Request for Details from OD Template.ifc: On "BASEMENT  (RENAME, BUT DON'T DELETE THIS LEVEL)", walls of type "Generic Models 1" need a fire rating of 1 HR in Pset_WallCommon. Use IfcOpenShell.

First a look at what the model holds.

```python
import ifcopenshell
import ifcopenshell.util.element

model = ifcopenshell.open("Details from OD Template.ifc")
print(model.schema)
storey = next(s for s in model.by_type("IfcBuildingStorey") if s.Name == "BASEMENT  (RENAME, BUT DON'T DELETE THIS LEVEL)")
walls = [e for e in ifcopenshell.util.element.get_decomposition(storey) if e.is_a("IfcWall")]
seen = {}
for e in walls:
    element_type = ifcopenshell.util.element.get_type(e)
    key = (element_type.Name if element_type != e and element_type else None, ifcopenshell.util.element.get_pset(e, "Pset_WallCommon", "FireRating"))
    seen[key] = seen.get(key, 0) + 1
for (name, value), count in sorted(seen.items(), key=str):
    print(count, "x", name, "|", value)
```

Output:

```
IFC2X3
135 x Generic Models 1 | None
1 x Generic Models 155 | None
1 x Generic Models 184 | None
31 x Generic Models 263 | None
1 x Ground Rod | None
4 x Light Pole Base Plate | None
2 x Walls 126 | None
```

```python
import ifcopenshell
import ifcopenshell.api.pset
import ifcopenshell.util.element

model = ifcopenshell.open("Details from OD Template.ifc")

storey = next(s for s in model.by_type("IfcBuildingStorey") if s.Name == "BASEMENT  (RENAME, BUT DON'T DELETE THIS LEVEL)")
walls = [e for e in ifcopenshell.util.element.get_decomposition(storey) if e.is_a("IfcWall")]

count = 0
for e in walls:
    element_type = ifcopenshell.util.element.get_type(e)
    if element_type in (None, e) or element_type.Name != "Generic Models 1":
        continue
    # add_pset returns the element's existing set when there is one.
    pset = ifcopenshell.api.pset.add_pset(model, product=e, name="Pset_WallCommon")
    ifcopenshell.api.pset.edit_pset(model, pset=pset, properties={"FireRating": "1 HR"})
    count += 1

print(count, "walls updated")

model.write("Details from OD Template_v2.ifc")
```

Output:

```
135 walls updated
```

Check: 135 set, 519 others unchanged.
